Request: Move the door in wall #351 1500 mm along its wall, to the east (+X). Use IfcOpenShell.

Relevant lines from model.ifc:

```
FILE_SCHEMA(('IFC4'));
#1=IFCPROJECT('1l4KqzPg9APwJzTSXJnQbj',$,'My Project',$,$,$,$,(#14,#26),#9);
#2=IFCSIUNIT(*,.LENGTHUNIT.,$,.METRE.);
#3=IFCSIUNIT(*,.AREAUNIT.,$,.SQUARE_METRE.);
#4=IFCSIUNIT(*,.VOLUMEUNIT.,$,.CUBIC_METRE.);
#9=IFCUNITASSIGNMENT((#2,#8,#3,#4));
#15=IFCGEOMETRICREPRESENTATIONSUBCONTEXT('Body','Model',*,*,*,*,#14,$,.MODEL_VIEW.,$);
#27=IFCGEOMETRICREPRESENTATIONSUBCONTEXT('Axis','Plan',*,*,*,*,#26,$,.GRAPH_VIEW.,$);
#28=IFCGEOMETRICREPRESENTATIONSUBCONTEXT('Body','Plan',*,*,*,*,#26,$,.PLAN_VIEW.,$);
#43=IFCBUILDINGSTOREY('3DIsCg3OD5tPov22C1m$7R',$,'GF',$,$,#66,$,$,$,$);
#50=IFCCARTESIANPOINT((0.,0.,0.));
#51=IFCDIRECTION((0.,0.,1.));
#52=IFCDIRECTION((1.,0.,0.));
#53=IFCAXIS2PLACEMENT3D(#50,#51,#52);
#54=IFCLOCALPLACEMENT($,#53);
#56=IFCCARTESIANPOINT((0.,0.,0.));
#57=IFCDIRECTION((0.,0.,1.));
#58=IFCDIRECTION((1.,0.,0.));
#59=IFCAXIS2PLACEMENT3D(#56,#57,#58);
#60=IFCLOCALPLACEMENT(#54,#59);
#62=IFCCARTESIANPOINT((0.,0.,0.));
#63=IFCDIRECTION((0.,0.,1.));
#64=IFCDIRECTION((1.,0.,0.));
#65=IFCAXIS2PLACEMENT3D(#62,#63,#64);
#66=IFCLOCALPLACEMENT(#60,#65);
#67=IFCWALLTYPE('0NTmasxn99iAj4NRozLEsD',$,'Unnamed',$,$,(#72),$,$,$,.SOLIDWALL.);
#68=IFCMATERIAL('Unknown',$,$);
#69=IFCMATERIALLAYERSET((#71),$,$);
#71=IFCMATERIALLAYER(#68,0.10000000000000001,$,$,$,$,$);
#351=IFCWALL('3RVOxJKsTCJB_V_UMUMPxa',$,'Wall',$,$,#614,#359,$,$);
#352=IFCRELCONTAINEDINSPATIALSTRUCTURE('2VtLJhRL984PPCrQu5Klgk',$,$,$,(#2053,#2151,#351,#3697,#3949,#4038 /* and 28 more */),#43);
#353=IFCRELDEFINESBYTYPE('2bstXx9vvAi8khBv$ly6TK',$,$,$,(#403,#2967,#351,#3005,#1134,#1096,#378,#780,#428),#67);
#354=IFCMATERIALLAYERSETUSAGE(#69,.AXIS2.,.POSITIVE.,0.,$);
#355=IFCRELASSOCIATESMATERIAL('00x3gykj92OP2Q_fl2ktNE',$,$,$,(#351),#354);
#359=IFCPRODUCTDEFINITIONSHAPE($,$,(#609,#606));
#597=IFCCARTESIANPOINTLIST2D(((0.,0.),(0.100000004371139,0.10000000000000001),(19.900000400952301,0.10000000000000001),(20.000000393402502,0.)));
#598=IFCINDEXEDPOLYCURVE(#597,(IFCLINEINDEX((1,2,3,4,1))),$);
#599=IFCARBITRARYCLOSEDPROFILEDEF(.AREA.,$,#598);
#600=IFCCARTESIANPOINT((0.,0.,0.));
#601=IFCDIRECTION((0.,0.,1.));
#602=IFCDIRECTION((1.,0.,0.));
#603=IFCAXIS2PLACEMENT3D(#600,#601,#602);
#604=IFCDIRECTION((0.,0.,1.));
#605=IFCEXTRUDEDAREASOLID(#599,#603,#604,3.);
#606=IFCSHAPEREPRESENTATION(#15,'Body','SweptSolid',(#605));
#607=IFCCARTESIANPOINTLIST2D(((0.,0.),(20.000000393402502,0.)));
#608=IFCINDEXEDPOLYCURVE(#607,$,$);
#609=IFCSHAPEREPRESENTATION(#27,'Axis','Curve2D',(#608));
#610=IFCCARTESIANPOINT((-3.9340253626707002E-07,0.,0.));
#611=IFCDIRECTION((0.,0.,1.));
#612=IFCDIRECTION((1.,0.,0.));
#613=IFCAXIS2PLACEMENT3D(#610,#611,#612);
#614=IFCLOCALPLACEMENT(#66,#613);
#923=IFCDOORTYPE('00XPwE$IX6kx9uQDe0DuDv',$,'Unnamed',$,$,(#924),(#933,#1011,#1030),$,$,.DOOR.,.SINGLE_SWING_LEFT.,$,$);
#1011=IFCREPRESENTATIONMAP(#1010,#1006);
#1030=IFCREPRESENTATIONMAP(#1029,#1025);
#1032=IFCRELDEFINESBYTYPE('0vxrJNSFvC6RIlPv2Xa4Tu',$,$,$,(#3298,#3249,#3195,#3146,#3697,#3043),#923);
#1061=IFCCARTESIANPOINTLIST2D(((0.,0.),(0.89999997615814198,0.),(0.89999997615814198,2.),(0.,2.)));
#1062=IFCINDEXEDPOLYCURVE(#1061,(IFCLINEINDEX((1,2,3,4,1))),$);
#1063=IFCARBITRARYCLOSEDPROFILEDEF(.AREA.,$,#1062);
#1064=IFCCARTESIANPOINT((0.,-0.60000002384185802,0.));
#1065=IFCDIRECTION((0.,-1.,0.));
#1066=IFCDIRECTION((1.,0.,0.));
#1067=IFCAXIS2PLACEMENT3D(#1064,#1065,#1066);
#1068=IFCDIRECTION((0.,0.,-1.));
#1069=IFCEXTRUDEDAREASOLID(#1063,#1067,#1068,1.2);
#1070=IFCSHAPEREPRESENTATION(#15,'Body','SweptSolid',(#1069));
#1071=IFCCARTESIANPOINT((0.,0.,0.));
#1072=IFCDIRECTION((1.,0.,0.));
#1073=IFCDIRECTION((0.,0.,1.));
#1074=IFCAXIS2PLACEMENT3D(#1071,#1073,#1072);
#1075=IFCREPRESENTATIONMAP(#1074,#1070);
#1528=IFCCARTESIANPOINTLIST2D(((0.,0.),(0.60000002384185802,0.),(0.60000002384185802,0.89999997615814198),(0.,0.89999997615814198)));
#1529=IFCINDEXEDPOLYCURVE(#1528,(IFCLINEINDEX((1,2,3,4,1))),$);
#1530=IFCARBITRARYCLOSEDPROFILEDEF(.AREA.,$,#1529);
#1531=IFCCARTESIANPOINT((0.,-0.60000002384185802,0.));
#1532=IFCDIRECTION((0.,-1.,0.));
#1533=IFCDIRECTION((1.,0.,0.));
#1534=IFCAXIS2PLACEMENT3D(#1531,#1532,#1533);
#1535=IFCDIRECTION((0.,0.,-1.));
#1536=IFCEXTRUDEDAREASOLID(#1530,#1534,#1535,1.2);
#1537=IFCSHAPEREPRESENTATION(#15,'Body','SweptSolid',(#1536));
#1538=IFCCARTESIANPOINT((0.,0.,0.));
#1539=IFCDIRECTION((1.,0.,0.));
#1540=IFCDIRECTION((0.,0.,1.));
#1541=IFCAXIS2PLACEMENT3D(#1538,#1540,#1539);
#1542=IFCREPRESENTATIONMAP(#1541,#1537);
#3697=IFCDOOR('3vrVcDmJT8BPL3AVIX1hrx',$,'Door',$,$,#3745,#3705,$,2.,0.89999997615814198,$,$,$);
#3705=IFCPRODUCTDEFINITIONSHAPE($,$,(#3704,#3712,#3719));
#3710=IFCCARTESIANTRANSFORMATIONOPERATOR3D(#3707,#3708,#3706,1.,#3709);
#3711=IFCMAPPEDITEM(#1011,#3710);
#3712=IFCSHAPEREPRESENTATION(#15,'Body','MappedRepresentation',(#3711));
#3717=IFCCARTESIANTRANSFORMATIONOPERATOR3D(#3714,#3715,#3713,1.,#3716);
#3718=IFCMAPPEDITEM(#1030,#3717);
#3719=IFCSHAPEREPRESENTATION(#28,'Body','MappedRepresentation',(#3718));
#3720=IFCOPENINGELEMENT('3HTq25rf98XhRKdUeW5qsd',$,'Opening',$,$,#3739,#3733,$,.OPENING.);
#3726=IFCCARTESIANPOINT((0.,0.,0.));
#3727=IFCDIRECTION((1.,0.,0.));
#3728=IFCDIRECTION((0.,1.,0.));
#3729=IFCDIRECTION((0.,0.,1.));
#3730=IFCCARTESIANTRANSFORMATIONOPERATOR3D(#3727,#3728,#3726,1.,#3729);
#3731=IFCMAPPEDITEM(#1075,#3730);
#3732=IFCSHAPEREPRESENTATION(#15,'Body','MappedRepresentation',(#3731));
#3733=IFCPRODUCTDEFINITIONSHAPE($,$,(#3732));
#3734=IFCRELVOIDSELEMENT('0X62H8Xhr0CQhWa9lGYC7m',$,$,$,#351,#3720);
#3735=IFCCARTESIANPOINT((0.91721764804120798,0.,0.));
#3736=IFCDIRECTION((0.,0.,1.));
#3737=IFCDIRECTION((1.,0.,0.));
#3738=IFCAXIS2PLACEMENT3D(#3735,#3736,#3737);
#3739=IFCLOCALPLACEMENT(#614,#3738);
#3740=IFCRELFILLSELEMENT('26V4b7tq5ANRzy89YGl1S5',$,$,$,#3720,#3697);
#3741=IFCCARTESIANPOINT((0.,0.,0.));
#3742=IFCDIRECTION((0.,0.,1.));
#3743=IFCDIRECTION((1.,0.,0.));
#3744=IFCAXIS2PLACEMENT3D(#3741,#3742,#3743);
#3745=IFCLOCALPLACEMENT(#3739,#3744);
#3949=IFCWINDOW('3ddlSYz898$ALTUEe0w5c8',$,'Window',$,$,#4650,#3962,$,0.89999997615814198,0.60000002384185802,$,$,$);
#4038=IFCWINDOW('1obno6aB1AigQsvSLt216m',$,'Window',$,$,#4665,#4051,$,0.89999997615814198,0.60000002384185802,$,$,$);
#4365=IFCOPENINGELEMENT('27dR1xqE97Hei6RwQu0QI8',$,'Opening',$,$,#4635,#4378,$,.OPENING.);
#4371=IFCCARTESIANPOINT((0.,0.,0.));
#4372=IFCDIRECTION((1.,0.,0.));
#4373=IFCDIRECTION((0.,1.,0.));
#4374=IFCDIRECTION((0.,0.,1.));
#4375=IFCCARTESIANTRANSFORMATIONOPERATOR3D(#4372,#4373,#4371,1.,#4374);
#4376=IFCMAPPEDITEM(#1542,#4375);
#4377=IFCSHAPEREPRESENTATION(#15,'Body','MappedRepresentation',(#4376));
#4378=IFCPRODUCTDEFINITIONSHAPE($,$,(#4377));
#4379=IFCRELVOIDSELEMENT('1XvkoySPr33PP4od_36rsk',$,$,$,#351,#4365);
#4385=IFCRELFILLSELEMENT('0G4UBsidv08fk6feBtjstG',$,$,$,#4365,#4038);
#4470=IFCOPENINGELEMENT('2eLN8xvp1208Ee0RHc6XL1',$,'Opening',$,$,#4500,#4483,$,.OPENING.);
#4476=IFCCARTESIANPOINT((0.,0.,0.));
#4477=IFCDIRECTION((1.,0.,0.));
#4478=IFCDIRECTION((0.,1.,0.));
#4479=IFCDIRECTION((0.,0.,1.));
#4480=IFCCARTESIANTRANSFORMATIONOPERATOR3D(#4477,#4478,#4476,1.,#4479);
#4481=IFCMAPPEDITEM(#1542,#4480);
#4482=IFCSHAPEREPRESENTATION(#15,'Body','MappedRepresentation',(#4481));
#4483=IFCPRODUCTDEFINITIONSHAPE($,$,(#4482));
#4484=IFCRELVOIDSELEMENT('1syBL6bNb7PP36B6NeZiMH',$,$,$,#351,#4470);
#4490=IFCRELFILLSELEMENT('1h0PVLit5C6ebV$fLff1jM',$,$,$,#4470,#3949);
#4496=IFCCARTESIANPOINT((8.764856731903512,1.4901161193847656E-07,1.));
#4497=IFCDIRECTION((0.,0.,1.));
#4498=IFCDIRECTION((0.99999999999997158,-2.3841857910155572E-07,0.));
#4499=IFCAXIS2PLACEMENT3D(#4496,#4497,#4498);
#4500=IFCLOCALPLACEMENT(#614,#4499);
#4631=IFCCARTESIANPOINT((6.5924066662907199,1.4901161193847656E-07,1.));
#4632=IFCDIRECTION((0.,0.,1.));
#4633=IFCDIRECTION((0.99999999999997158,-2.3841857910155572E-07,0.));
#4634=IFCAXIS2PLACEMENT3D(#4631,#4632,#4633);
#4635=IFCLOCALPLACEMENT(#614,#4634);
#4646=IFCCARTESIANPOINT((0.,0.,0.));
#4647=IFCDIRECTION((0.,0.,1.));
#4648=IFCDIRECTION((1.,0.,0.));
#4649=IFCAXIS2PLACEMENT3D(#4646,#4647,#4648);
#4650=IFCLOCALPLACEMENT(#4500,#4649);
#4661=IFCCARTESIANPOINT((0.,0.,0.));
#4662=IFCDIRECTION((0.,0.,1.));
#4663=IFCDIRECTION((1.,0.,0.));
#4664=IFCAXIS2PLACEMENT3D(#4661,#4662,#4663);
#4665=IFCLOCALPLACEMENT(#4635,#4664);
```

```python
import ifcopenshell
import ifcopenshell.api.geometry
import ifcopenshell.util.placement

model = ifcopenshell.open("model.ifc")

door = model.by_guid("3vrVcDmJT8BPL3AVIX1hrx")
opening = door.FillsVoids[0].RelatingOpeningElement
wall = opening.VoidsElements[0].RelatingBuildingElement

wall_matrix = ifcopenshell.util.placement.get_local_placement(wall.ObjectPlacement)
shift = wall_matrix[:3, 0] * 1.5
before = ifcopenshell.util.placement.get_local_placement(door.ObjectPlacement)[:3, 3].copy()

# The door is placed relative to its opening, so it follows when the opening moves.
matrix = ifcopenshell.util.placement.get_local_placement(opening.ObjectPlacement)
matrix[:3, 3] += shift
ifcopenshell.api.geometry.edit_object_placement(
    model, product=opening, matrix=matrix, is_si=False, should_transform_children=True
)

after = ifcopenshell.util.placement.get_local_placement(door.ObjectPlacement)[:3, 3]
print("door moved by", (after - before).round(3) + 0.0)

model.write("model_updated.ifc")
```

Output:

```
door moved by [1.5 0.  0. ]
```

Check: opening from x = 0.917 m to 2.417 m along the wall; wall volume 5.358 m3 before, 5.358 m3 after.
